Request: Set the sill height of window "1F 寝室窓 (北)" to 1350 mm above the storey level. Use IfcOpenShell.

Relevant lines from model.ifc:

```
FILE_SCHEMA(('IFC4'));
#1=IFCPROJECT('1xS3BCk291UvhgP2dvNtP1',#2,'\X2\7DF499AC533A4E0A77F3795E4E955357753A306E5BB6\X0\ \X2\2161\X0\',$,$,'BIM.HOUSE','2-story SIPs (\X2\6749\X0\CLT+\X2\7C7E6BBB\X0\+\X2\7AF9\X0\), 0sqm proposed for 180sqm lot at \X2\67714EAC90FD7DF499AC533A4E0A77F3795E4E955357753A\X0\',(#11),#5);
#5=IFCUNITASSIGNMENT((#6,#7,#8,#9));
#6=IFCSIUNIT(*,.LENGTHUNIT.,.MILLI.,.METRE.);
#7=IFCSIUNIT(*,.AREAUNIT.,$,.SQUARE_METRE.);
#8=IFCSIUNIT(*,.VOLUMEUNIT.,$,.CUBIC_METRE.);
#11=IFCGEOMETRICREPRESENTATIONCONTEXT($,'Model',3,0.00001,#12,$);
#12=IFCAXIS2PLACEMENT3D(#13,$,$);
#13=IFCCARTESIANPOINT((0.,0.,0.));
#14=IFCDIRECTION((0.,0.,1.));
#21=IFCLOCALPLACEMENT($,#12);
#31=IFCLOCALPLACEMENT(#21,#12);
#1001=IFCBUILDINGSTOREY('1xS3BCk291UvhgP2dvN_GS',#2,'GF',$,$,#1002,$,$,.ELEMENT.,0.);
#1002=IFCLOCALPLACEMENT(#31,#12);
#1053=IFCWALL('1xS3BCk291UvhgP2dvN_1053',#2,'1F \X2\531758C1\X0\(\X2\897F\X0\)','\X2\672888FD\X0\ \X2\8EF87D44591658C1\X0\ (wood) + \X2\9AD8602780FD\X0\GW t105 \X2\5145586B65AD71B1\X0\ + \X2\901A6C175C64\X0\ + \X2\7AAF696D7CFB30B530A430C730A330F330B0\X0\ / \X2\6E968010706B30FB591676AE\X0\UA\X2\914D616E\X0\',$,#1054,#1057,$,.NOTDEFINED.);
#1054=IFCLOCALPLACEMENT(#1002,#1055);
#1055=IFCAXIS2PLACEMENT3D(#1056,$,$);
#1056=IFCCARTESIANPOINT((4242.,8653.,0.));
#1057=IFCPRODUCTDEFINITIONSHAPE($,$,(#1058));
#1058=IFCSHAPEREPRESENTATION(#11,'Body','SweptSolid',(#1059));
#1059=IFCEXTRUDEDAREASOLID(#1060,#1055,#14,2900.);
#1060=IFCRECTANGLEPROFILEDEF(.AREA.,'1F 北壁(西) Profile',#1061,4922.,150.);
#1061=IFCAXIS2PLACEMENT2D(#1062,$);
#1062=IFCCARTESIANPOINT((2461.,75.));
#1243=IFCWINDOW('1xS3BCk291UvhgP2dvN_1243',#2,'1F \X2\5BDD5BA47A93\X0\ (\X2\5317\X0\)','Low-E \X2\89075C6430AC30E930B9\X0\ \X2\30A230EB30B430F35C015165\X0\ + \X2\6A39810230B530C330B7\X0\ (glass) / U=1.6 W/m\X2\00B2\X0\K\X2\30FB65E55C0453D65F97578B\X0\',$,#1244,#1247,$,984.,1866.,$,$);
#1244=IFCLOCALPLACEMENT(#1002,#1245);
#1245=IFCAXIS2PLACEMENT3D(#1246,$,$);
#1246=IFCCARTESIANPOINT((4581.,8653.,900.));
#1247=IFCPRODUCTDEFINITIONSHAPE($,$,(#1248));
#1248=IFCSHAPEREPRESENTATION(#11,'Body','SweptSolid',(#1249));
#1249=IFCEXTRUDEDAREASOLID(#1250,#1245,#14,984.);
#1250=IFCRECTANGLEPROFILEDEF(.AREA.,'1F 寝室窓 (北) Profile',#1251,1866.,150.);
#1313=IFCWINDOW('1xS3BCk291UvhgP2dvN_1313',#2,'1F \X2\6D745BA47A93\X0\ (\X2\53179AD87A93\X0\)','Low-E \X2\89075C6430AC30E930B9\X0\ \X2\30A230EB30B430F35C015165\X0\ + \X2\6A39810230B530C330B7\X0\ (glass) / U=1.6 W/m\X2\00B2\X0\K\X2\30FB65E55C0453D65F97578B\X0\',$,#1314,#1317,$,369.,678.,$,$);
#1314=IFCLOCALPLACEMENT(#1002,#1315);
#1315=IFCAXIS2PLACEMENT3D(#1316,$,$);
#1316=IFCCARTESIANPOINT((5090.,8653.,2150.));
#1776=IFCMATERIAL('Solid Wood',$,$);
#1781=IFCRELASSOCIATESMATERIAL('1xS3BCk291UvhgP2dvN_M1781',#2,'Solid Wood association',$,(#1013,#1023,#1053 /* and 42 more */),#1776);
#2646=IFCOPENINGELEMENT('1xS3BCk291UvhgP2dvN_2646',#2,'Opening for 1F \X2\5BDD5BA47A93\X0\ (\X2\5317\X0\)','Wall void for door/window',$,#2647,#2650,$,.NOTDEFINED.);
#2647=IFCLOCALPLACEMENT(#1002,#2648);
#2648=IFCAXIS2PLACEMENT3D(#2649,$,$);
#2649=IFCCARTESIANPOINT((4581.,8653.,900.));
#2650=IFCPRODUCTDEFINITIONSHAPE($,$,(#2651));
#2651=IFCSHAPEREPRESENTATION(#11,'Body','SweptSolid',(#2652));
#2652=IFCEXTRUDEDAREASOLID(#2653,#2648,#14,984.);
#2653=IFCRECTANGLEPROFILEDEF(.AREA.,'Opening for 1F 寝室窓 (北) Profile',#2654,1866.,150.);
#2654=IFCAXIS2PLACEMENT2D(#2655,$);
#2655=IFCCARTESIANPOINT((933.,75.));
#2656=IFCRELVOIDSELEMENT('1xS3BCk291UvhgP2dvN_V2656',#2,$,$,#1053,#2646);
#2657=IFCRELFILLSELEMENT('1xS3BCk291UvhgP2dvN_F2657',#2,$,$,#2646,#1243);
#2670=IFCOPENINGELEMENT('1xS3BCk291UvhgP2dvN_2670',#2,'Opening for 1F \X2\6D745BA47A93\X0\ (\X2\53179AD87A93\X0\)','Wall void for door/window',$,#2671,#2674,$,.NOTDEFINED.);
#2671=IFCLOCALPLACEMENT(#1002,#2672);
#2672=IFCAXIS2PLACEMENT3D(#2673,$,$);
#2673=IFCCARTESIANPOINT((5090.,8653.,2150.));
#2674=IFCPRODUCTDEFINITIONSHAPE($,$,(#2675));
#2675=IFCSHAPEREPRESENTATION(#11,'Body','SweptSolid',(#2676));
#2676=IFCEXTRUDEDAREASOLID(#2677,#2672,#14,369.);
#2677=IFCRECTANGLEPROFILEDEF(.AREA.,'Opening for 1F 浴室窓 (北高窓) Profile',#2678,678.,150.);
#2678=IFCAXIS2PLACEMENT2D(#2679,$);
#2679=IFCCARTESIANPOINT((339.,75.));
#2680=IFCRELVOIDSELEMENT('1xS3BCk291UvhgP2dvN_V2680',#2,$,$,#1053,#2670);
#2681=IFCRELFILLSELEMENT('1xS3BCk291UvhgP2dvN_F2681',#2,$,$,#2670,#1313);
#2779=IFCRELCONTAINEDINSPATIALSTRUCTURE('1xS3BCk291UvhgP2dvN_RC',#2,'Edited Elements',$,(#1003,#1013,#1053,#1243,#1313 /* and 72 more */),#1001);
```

```python
import numpy as np
import ifcopenshell
import ifcopenshell.api.geometry
import ifcopenshell.geom
import ifcopenshell.util.element
import ifcopenshell.util.placement
import ifcopenshell.util.shape
import ifcopenshell.util.unit

model = ifcopenshell.open("model.ifc")
unit_scale = ifcopenshell.util.unit.calculate_unit_scale(model)

window = model.by_guid("1xS3BCk291UvhgP2dvN_1243")
opening = window.FillsVoids[0].RelatingOpeningElement
storey = ifcopenshell.util.element.get_container(window, ifc_class="IfcBuildingStorey")
level = ifcopenshell.util.placement.get_local_placement(storey.ObjectPlacement)[2, 3]

# The opening's origin need not be at the sill, so measure its lowest point.
shape = ifcopenshell.geom.create_shape(ifcopenshell.geom.settings(), opening)
bottom = ifcopenshell.util.shape.get_shape_bottom_elevation(shape, shape.geometry) / unit_scale
dz = level + 1350.0 - bottom

shift = np.array([0.0, 0.0, dz])
# The window is not placed relative to its opening, so move both.
for product in (opening, window):
    matrix = ifcopenshell.util.placement.get_local_placement(product.ObjectPlacement)
    matrix[:3, 3] += shift
    ifcopenshell.api.geometry.edit_object_placement(model, product=product, matrix=matrix, is_si=False)

print(f"moved by {dz * unit_scale:+.3f} m")

model.write("model_updated.ifc")
```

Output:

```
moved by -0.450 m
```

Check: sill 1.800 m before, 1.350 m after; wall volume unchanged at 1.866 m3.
